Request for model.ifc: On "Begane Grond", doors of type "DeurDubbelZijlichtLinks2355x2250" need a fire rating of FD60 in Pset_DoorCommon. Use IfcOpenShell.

First a look at what the model holds.

```python
import ifcopenshell
import ifcopenshell.util.element

model = ifcopenshell.open("model.ifc")
print(model.schema)
storey = next(s for s in model.by_type("IfcBuildingStorey") if s.Name == "Begane Grond")
doors = [e for e in ifcopenshell.util.element.get_decomposition(storey) if e.is_a("IfcDoor")]
seen = {}
for e in doors:
    element_type = ifcopenshell.util.element.get_type(e)
    key = (element_type.Name if element_type != e and element_type else None, ifcopenshell.util.element.get_pset(e, "Pset_DoorCommon", "FireRating"))
    seen[key] = seen.get(key, 0) + 1
for (name, value), count in sorted(seen.items(), key=str):
    print(count, "x", name, "|", value)
```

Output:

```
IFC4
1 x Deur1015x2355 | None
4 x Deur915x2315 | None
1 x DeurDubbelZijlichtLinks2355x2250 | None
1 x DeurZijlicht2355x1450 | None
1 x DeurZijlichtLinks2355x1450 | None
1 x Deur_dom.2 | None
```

```python
import ifcopenshell
import ifcopenshell.api.pset
import ifcopenshell.util.element

model = ifcopenshell.open("model.ifc")

storey = next(s for s in model.by_type("IfcBuildingStorey") if s.Name == "Begane Grond")
doors = [e for e in ifcopenshell.util.element.get_decomposition(storey) if e.is_a("IfcDoor")]

count = 0
for e in doors:
    element_type = ifcopenshell.util.element.get_type(e)
    if element_type in (None, e) or element_type.Name != "DeurDubbelZijlichtLinks2355x2250":
        continue
    # add_pset returns the element's existing set when there is one.
    pset = ifcopenshell.api.pset.add_pset(model, product=e, name="Pset_DoorCommon")
    ifcopenshell.api.pset.edit_pset(model, pset=pset, properties={"FireRating": "FD60"})
    count += 1

print(count, "doors updated")

model.write("model-out.ifc")
```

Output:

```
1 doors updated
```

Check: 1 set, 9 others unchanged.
